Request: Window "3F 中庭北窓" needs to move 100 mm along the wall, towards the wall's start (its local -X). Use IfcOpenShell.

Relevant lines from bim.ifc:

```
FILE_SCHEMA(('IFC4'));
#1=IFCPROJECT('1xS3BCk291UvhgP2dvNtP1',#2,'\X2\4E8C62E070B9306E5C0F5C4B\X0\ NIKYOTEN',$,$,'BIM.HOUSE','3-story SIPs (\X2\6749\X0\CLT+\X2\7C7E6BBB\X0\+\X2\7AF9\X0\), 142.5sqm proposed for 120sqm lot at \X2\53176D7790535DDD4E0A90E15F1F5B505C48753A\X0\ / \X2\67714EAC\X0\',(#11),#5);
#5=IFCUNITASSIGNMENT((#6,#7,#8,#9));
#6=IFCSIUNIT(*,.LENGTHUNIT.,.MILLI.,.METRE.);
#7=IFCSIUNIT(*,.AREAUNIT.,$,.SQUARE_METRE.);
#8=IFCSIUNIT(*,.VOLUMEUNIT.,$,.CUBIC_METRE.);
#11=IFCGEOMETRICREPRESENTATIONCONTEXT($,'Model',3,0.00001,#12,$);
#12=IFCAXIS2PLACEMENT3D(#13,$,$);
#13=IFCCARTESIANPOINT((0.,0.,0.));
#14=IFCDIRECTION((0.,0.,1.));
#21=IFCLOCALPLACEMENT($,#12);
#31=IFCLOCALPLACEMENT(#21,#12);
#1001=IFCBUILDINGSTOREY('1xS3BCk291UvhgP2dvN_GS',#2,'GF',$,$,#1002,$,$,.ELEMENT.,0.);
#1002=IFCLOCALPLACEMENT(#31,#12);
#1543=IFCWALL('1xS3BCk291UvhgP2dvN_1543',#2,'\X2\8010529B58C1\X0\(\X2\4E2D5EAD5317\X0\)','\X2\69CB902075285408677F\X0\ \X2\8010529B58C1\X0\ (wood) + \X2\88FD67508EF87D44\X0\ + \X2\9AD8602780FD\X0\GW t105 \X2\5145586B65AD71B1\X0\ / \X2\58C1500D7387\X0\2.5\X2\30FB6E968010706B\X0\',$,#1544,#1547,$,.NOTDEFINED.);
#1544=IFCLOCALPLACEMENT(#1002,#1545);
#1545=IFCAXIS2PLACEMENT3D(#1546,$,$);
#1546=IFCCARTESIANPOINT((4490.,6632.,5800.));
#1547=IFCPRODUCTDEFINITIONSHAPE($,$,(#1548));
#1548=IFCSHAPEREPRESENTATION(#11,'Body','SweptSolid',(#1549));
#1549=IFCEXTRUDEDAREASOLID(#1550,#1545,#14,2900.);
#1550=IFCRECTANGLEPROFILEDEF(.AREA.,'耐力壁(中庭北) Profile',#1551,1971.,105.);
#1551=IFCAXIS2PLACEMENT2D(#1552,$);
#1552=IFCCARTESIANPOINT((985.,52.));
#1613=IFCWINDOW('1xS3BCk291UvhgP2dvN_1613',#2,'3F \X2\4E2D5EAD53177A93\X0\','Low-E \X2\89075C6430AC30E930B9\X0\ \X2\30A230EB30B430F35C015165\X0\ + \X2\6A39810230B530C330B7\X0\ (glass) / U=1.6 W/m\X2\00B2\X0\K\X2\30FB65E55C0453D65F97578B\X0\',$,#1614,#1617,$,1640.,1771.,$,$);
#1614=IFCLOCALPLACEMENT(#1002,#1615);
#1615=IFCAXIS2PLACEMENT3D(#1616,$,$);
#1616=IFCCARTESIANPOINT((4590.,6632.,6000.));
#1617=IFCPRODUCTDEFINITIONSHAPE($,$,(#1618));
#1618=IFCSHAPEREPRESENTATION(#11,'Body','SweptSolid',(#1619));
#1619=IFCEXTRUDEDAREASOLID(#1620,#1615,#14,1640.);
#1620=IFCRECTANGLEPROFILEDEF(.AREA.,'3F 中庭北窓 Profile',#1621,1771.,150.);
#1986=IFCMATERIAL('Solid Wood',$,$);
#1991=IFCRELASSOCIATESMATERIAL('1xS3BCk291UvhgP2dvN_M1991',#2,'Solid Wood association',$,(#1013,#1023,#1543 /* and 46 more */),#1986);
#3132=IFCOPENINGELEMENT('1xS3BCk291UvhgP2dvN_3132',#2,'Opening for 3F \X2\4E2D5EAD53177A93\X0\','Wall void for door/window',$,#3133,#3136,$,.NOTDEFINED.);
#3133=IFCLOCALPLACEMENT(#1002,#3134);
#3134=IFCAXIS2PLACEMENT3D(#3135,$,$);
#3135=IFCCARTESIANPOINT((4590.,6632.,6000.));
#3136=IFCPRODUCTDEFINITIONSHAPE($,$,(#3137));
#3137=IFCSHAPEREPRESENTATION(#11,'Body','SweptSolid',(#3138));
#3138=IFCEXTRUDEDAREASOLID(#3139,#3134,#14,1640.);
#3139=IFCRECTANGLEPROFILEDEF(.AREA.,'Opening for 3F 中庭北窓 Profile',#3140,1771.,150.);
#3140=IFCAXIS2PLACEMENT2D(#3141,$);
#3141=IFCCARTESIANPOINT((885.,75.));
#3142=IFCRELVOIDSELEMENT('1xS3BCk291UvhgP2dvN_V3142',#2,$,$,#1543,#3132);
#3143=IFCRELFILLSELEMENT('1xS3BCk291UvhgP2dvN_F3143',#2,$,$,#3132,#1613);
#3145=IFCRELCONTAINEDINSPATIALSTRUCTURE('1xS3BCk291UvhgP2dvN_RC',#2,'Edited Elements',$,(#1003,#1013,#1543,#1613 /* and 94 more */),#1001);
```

```python
import ifcopenshell
import ifcopenshell.api.geometry
import ifcopenshell.util.placement
import ifcopenshell.util.unit

model = ifcopenshell.open("bim.ifc")
unit_scale = ifcopenshell.util.unit.calculate_unit_scale(model)

window = model.by_id(1613)
opening = window.FillsVoids[0].RelatingOpeningElement
wall = opening.VoidsElements[0].RelatingBuildingElement

wall_matrix = ifcopenshell.util.placement.get_local_placement(wall.ObjectPlacement)
shift = wall_matrix[:3, 0] * -0.1 / unit_scale
before = ifcopenshell.util.placement.get_local_placement(window.ObjectPlacement)[:3, 3].copy()

# The window is not placed relative to its opening, so move both.
for product in (opening, window):
    matrix = ifcopenshell.util.placement.get_local_placement(product.ObjectPlacement)
    matrix[:3, 3] += shift
    ifcopenshell.api.geometry.edit_object_placement(model, product=product, matrix=matrix, is_si=False)

after = ifcopenshell.util.placement.get_local_placement(window.ObjectPlacement)[:3, 3]
print("window moved by", (after - before).round(3) + 0.0)

model.write("bim_updated.ifc")
```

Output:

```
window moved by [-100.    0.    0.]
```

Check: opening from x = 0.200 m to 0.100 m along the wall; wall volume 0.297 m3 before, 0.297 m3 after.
